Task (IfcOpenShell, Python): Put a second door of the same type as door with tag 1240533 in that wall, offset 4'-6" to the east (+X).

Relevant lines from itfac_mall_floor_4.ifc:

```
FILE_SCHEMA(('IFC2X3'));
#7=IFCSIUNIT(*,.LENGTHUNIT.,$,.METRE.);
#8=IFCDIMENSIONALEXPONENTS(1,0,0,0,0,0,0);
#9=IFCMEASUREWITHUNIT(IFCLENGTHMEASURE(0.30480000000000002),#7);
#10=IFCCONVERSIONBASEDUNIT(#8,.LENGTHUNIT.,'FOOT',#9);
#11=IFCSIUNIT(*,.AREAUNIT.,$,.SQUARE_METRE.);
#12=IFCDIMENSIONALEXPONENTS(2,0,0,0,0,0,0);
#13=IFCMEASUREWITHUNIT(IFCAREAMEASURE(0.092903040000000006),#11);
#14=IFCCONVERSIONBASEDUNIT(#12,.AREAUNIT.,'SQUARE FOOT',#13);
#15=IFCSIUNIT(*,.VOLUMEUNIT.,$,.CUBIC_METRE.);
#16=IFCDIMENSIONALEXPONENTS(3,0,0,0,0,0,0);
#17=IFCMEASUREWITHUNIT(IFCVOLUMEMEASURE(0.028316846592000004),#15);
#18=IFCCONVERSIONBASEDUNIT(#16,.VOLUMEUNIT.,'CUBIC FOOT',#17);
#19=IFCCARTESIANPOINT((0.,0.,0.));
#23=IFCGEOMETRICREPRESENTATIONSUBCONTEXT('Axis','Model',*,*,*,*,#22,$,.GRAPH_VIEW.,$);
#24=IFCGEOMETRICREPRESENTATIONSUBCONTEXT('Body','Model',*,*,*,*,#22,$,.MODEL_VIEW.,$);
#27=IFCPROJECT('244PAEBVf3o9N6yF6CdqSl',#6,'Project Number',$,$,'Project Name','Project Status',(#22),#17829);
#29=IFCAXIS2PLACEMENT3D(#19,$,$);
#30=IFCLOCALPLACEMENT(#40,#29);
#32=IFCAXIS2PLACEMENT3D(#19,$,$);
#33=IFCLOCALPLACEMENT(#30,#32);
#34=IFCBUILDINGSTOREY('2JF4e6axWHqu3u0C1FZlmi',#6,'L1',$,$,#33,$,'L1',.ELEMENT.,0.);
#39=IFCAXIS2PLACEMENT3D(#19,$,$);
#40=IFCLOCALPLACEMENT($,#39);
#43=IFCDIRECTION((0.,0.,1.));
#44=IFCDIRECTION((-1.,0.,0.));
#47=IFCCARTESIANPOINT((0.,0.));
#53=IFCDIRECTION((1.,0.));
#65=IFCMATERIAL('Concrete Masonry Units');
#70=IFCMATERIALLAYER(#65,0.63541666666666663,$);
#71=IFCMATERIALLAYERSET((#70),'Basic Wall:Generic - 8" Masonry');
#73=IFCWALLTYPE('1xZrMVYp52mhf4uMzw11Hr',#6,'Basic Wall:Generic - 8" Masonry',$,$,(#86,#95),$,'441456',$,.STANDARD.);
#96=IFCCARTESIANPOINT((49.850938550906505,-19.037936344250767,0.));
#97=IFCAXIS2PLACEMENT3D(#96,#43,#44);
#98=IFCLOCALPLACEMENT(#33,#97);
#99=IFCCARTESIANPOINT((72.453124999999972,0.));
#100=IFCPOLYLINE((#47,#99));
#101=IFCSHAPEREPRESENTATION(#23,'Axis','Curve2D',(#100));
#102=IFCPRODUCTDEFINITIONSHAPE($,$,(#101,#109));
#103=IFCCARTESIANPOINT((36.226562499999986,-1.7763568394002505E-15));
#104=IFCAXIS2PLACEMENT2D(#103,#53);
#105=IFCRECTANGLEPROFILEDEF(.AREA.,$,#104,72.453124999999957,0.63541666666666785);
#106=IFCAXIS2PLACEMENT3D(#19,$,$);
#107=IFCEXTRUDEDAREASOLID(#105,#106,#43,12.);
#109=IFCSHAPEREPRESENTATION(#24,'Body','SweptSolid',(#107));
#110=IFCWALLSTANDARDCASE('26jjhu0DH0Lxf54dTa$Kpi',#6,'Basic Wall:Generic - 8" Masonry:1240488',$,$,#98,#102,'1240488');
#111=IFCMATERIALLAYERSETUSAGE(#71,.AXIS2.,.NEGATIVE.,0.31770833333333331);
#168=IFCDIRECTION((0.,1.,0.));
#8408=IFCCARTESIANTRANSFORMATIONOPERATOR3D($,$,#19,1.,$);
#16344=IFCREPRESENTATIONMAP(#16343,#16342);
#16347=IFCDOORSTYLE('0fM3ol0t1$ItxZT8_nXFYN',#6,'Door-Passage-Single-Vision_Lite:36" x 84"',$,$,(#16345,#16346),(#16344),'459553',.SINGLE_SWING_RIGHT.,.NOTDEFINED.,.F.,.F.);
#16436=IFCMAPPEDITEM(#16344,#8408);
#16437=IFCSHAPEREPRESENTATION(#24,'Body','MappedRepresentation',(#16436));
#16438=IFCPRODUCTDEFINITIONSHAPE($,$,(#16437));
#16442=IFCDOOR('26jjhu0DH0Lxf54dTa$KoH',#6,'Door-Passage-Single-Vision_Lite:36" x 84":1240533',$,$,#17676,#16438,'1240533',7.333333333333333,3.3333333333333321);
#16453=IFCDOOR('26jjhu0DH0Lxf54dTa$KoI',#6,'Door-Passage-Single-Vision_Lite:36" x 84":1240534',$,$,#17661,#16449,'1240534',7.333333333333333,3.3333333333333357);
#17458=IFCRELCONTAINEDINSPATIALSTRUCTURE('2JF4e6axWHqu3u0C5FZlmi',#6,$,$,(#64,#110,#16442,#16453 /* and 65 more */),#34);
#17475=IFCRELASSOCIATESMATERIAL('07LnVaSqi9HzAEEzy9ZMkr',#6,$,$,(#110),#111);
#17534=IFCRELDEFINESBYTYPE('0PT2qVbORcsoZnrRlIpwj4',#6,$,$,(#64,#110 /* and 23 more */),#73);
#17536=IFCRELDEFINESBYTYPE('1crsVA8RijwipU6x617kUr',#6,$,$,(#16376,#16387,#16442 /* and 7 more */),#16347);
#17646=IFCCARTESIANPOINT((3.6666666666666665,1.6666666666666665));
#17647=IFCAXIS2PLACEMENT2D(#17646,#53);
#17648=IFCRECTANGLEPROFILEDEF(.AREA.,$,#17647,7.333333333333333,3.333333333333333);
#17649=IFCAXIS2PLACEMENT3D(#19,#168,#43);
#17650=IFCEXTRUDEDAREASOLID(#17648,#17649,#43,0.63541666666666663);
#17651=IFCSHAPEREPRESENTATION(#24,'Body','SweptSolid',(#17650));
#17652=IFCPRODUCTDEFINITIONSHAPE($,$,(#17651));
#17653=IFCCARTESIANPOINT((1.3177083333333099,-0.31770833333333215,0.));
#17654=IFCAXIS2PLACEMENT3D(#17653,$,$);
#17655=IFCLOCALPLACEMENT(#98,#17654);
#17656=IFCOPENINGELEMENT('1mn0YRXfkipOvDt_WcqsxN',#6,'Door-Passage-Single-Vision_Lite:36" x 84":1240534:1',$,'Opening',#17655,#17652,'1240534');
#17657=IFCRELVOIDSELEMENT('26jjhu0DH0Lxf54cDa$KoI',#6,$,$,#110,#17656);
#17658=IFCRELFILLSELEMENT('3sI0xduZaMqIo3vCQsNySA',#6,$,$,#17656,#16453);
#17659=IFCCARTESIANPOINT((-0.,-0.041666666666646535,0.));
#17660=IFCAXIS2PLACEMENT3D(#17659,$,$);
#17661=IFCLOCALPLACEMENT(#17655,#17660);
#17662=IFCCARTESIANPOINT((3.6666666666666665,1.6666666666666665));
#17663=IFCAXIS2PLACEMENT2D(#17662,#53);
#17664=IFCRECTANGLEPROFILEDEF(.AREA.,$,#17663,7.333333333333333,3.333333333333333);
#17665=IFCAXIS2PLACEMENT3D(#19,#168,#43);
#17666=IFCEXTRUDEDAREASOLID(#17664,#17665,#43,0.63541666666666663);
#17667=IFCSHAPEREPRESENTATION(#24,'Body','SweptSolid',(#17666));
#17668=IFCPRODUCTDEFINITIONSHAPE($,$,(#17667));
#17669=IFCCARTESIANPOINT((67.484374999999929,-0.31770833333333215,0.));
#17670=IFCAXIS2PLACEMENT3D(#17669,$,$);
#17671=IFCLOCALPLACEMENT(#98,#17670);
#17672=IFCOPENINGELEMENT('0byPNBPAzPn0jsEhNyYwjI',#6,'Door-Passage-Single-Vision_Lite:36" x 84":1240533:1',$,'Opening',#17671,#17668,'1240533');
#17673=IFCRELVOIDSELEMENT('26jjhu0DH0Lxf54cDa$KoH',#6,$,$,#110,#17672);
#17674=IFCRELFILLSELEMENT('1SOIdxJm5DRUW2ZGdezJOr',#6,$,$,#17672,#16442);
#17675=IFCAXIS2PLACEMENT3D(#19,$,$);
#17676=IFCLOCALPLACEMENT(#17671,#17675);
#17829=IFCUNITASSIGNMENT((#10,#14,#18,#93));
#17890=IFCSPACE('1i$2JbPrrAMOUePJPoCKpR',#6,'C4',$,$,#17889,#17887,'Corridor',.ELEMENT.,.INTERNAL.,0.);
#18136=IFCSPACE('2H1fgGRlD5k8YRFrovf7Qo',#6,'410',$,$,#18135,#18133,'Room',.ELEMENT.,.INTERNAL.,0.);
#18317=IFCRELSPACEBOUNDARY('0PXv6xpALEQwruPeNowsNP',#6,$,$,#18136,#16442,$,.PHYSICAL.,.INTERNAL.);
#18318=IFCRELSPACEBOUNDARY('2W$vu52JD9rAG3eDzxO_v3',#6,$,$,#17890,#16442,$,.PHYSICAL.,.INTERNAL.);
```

```python
import ifcopenshell
import ifcopenshell.api.feature
import ifcopenshell.api.geometry
import ifcopenshell.api.root
import ifcopenshell.geom
import ifcopenshell.util.element
import ifcopenshell.util.placement
import ifcopenshell.util.shape
import ifcopenshell.util.unit

model = ifcopenshell.open("itfac_mall_floor_4.ifc")
unit_scale = ifcopenshell.util.unit.calculate_unit_scale(model)
settings = ifcopenshell.geom.settings()


def volume(element):
    """Net volume in cubic metres, openings subtracted."""
    shape = ifcopenshell.geom.create_shape(settings, element)
    return ifcopenshell.util.shape.get_volume(shape.geometry)


def reuse_history(source, copy):
    """copy_class also copies each property set's owner history, people and application; keep the originals."""
    for rel in copy.IsDefinedBy:
        if rel.is_a("IfcRelDefinesByProperties") and (history := rel.RelatingPropertyDefinition.OwnerHistory):
            rel.RelatingPropertyDefinition.OwnerHistory = source.OwnerHistory
            ifcopenshell.util.element.remove_deep2(model, history)


door = model.by_guid("26jjhu0DH0Lxf54dTa$KoH")
opening = door.FillsVoids[0].RelatingOpeningElement
wall = opening.VoidsElements[0].RelatingBuildingElement
before = volume(wall)
shift = ifcopenshell.util.placement.get_local_placement(wall.ObjectPlacement)[:3, 0] * -54 * 0.0254 / unit_scale

# copy_class copies the void relationship, type, container and properties, but no geometry.
new_opening = ifcopenshell.api.root.copy_class(model, product=opening)
new_opening.Representation = ifcopenshell.util.element.copy_deep(
    model, opening.Representation, exclude=["IfcGeometricRepresentationContext", "IfcRepresentationMap"]
)
new_opening.Name = 'Door-Passage-Single-Vision_Lite:36" x 84"'
new_opening.Tag = None
new_door = ifcopenshell.api.root.copy_class(model, product=door)
new_door.Representation = ifcopenshell.util.element.copy_deep(
    model, door.Representation, exclude=["IfcGeometricRepresentationContext", "IfcRepresentationMap"]
)
new_door.Name = 'Door-Passage-Single-Vision_Lite:36" x 84"'
new_door.Tag = None
reuse_history(door, new_door)
fills = ifcopenshell.api.feature.add_filling(model, opening=new_opening, element=new_door)
fills.OwnerHistory = new_door.OwnerHistory  # required in IFC2X3

for old, new in ((opening, new_opening), (door, new_door)):
    matrix = ifcopenshell.util.placement.get_local_placement(old.ObjectPlacement)
    matrix[:3, 3] += shift
    ifcopenshell.api.geometry.edit_object_placement(model, product=new, matrix=matrix, is_si=False)

after = volume(wall)

print(f"wall volume {before:.3f} -> {after:.3f} m3")

model.write("itfac_mall_floor_4-out.ifc")
```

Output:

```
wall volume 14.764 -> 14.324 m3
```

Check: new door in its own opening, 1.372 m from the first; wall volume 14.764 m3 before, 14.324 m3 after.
